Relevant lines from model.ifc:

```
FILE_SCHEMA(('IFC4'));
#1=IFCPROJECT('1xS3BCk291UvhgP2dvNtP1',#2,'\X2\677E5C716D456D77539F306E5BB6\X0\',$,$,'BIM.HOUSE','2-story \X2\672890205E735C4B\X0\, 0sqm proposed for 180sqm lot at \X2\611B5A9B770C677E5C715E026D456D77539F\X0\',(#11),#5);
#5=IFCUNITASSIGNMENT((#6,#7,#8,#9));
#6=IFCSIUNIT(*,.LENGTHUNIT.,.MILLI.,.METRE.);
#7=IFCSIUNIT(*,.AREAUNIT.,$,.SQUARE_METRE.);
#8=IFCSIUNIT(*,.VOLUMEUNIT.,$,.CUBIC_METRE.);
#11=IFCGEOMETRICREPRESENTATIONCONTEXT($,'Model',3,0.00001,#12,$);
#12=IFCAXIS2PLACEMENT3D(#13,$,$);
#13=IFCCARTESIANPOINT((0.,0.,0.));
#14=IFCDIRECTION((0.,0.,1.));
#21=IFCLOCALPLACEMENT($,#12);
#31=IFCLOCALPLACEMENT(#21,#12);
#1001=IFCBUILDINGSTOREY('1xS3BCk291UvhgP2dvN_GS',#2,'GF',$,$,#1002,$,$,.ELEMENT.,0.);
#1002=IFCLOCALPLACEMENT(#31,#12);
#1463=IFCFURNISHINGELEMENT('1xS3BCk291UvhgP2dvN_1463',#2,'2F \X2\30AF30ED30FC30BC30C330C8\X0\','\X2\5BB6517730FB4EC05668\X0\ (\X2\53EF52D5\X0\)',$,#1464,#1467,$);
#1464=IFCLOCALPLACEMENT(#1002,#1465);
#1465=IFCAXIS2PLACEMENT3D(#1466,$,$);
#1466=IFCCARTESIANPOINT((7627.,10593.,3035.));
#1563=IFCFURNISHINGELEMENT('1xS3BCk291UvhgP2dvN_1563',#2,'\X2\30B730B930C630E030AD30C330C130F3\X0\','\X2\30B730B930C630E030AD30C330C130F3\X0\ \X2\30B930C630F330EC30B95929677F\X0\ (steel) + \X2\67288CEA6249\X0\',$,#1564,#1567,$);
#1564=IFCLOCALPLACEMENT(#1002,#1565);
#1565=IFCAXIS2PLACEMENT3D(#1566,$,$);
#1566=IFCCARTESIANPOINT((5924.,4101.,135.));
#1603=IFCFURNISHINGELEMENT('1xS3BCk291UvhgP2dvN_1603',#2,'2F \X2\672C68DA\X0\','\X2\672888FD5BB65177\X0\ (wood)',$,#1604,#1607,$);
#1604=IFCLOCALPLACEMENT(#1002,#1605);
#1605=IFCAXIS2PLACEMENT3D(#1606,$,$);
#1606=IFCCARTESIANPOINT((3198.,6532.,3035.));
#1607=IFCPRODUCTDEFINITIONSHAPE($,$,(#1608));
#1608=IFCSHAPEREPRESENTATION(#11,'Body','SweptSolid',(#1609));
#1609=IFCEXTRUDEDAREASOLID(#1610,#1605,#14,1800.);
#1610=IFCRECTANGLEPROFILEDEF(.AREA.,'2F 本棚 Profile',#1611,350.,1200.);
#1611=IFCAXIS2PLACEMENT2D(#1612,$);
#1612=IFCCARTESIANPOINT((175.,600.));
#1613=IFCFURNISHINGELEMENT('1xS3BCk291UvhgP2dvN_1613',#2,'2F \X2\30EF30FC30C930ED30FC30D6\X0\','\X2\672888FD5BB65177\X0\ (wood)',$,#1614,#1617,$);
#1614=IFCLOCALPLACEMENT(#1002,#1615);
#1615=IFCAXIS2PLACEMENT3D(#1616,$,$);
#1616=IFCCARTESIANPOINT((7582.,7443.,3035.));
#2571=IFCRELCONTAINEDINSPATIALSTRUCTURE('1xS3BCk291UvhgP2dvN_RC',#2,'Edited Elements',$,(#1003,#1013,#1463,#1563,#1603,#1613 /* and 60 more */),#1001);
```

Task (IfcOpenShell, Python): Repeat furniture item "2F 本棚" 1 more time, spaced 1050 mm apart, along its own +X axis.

```python
import ifcopenshell
import ifcopenshell.api.geometry
import ifcopenshell.api.root
import ifcopenshell.util.element
import ifcopenshell.util.placement

model = ifcopenshell.open("model.ifc")


def reuse_history(source, copy):
    """copy_class also copies each property set's owner history, people and application; keep the originals."""
    for rel in copy.IsDefinedBy:
        if rel.is_a("IfcRelDefinesByProperties") and (history := rel.RelatingPropertyDefinition.OwnerHistory):
            rel.RelatingPropertyDefinition.OwnerHistory = source.OwnerHistory
            ifcopenshell.util.element.remove_deep2(model, history)


source = model.by_guid("1xS3BCk291UvhgP2dvN_1603")
base = ifcopenshell.util.placement.get_local_placement(source.ObjectPlacement)
step = base[:3, 0] * 1050.0

for i in range(1, 2):
    copy = ifcopenshell.api.root.copy_class(model, product=source)
    copy.Representation = ifcopenshell.util.element.copy_deep(
        model, source.Representation, exclude=["IfcGeometricRepresentationContext", "IfcRepresentationMap"]
    )
    reuse_history(source, copy)
    matrix = base.copy()
    matrix[:3, 3] += i * step
    print("added at", matrix[:3, 3].round(3) + 0.0)
    ifcopenshell.api.geometry.edit_object_placement(model, product=copy, matrix=matrix, is_si=False)

model.write("model_v2.ifc")
```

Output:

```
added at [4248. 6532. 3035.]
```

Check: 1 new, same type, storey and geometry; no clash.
